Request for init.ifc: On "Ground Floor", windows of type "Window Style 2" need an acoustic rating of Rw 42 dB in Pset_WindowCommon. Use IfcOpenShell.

First a look at what the model holds.

```python
import ifcopenshell
import ifcopenshell.util.element

model = ifcopenshell.open("init.ifc")
print(model.schema)
storey = next(s for s in model.by_type("IfcBuildingStorey") if s.Name == "Ground Floor")
windows = [e for e in ifcopenshell.util.element.get_decomposition(storey) if e.is_a("IfcWindow")]
seen = {}
for e in windows:
    element_type = ifcopenshell.util.element.get_type(e)
    key = (element_type.Name if element_type != e and element_type else None, ifcopenshell.util.element.get_pset(e, "Pset_WindowCommon", "AcousticRating"))
    seen[key] = seen.get(key, 0) + 1
for (name, value), count in sorted(seen.items(), key=str):
    print(count, "x", name, "|", value)
```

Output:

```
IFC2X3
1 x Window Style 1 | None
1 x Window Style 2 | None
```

```python
import ifcopenshell
import ifcopenshell.api.pset
import ifcopenshell.util.element

model = ifcopenshell.open("init.ifc")

storey = next(s for s in model.by_type("IfcBuildingStorey") if s.Name == "Ground Floor")
windows = [e for e in ifcopenshell.util.element.get_decomposition(storey) if e.is_a("IfcWindow")]

count = 0
for e in windows:
    element_type = ifcopenshell.util.element.get_type(e)
    if element_type in (None, e) or element_type.Name != "Window Style 2":
        continue
    # add_pset returns the element's existing set when there is one.
    pset = ifcopenshell.api.pset.add_pset(model, product=e, name="Pset_WindowCommon")
    ifcopenshell.api.pset.edit_pset(model, pset=pset, properties={"AcousticRating": "Rw 42 dB"})
    count += 1

print(count, "windows updated")

model.write("init_rev.ifc")
```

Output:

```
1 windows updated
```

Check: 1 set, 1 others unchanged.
